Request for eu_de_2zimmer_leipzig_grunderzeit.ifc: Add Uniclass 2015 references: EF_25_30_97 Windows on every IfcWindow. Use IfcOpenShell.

First a look at what the model holds.

```python
import ifcopenshell

model = ifcopenshell.open("eu_de_2zimmer_leipzig_grunderzeit.ifc")
print(model.schema)
print("classifications:", [c.Name for c in model.by_type("IfcClassification")])
for ifc_class in ("IfcDoor", "IfcRoof", "IfcStair", "IfcWall", "IfcWindow"):
    print(ifc_class, len(model.by_type(ifc_class)))
```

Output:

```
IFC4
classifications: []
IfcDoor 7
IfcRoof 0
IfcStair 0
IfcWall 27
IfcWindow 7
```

```python
import ifcopenshell
import ifcopenshell.api.classification

model = ifcopenshell.open("eu_de_2zimmer_leipzig_grunderzeit.ifc")

system = ifcopenshell.api.classification.add_classification(model, classification="Uniclass 2015")

codes = {
    "IfcWindow": ("EF_25_30_97", "Windows"),
}
for ifc_class, (code, name) in codes.items():
    products = model.by_type(ifc_class)
    ifcopenshell.api.classification.add_reference(
        model, products=products, classification=system, identification=code, name=name
    )
    print(code, len(products))

model.write("eu_de_2zimmer_leipzig_grunderzeit_updated.ifc")
```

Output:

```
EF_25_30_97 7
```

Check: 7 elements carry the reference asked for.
